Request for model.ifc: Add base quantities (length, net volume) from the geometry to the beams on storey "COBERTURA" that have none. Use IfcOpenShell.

First a look at what the model holds.

```python
import ifcopenshell
import ifcopenshell.util.element
import ifcopenshell.util.unit

model = ifcopenshell.open("model.ifc")
print(model.schema)
for unit_type in ("LENGTHUNIT", "AREAUNIT", "VOLUMEUNIT"):
    print(unit_type, ifcopenshell.util.unit.calculate_unit_scale(model, unit_type))
storey = next(s for s in model.by_type("IfcBuildingStorey") if s.Name == "COBERTURA")
beams = [e for e in ifcopenshell.util.element.get_decomposition(storey) if e.is_a("IfcBeam")]
for e in sorted(beams, key=lambda e: e.id()):
    print(e.id(), e.is_a(), e.Name, list(ifcopenshell.util.element.get_psets(e, qtos_only=True)), sep=" | ")
```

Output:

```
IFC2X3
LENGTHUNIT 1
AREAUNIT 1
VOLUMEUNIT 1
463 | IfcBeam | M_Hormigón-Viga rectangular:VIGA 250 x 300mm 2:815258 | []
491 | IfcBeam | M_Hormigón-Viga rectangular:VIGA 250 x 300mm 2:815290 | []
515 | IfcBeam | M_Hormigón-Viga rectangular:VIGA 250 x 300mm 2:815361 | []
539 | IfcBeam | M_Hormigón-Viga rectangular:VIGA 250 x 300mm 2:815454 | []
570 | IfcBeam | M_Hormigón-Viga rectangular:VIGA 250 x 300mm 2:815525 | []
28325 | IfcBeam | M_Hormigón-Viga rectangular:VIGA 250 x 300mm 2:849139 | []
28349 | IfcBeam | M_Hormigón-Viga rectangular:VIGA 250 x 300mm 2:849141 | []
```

```python
import ifcopenshell
import ifcopenshell.api.pset
import ifcopenshell.geom
import ifcopenshell.util.element
import ifcopenshell.util.shape
import ifcopenshell.util.unit

model = ifcopenshell.open("model.ifc")
unit_scale = ifcopenshell.util.unit.calculate_unit_scale(model)
volume_scale = ifcopenshell.util.unit.calculate_unit_scale(model, "VOLUMEUNIT")
settings = ifcopenshell.geom.settings()

storey = next(s for s in model.by_type("IfcBuildingStorey") if s.Name == "COBERTURA")
beams = [e for e in ifcopenshell.util.element.get_decomposition(storey) if e.is_a("IfcBeam")]

for e in sorted(beams, key=lambda e: e.id()):
    if ifcopenshell.util.element.get_psets(e, qtos_only=True, should_inherit=False):
        continue
    # Geometry comes back in metres, in the element's own axes.
    shape = ifcopenshell.geom.create_shape(settings, e)
    values = {
        "Length": ifcopenshell.util.shape.get_max_xyz(shape.geometry) / unit_scale,
        "NetVolume": ifcopenshell.util.shape.get_volume(shape.geometry) / volume_scale,
    }
    qto = ifcopenshell.api.pset.add_qto(model, product=e, name="BaseQuantities")
    ifcopenshell.api.pset.edit_qto(model, qto=qto, properties=values)
    print(e.id(), {k: round(v, 3) for k, v in values.items()})

model.write("model_rev.ifc")
```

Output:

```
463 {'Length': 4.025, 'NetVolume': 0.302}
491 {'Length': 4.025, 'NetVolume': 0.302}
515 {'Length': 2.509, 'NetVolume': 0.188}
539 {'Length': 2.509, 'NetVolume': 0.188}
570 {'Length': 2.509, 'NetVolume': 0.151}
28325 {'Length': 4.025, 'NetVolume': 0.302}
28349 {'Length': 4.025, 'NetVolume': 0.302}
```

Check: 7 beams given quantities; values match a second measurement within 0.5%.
